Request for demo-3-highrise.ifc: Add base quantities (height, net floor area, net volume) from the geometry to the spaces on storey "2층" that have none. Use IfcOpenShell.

First a look at what the model holds.

```python
import ifcopenshell
import ifcopenshell.util.element
import ifcopenshell.util.unit

model = ifcopenshell.open("demo-3-highrise.ifc")
print(model.schema)
for unit_type in ("LENGTHUNIT", "AREAUNIT", "VOLUMEUNIT"):
    print(unit_type, ifcopenshell.util.unit.calculate_unit_scale(model, unit_type))
storey = next(s for s in model.by_type("IfcBuildingStorey") if s.Name == "2층")
spaces = [e for e in ifcopenshell.util.element.get_decomposition(storey) if e.is_a("IfcSpace")]
for e in sorted(spaces, key=lambda e: e.id()):
    print(e.id(), e.is_a(), e.Name, list(ifcopenshell.util.element.get_psets(e, qtos_only=True)), sep=" | ")
```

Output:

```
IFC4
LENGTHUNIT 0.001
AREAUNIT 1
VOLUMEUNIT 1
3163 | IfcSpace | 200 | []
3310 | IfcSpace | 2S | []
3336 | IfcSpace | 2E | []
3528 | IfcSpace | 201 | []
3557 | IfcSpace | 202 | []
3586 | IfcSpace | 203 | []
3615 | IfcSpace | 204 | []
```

```python
import ifcopenshell
import ifcopenshell.api.pset
import ifcopenshell.geom
import ifcopenshell.util.element
import ifcopenshell.util.shape
import ifcopenshell.util.unit

model = ifcopenshell.open("demo-3-highrise.ifc")
unit_scale = ifcopenshell.util.unit.calculate_unit_scale(model)
area_scale = ifcopenshell.util.unit.calculate_unit_scale(model, "AREAUNIT")
volume_scale = ifcopenshell.util.unit.calculate_unit_scale(model, "VOLUMEUNIT")
settings = ifcopenshell.geom.settings()

storey = next(s for s in model.by_type("IfcBuildingStorey") if s.Name == "2층")
spaces = [e for e in ifcopenshell.util.element.get_decomposition(storey) if e.is_a("IfcSpace")]

for e in sorted(spaces, key=lambda e: e.id()):
    if ifcopenshell.util.element.get_psets(e, qtos_only=True, should_inherit=False):
        continue
    # Geometry comes back in metres, in the element's own axes.
    shape = ifcopenshell.geom.create_shape(settings, e)
    values = {
        "Height": ifcopenshell.util.shape.get_z(shape.geometry) / unit_scale,
        "NetFloorArea": ifcopenshell.util.shape.get_footprint_area(shape.geometry) / area_scale,
        "NetVolume": ifcopenshell.util.shape.get_volume(shape.geometry) / volume_scale,
    }
    qto = ifcopenshell.api.pset.add_qto(model, product=e, name="Qto_SpaceBaseQuantities")
    ifcopenshell.api.pset.edit_qto(model, qto=qto, properties=values)
    print(e.id(), {k: round(v, 3) for k, v in values.items()})

model.write("demo-3-highrise_v2.ifc")
```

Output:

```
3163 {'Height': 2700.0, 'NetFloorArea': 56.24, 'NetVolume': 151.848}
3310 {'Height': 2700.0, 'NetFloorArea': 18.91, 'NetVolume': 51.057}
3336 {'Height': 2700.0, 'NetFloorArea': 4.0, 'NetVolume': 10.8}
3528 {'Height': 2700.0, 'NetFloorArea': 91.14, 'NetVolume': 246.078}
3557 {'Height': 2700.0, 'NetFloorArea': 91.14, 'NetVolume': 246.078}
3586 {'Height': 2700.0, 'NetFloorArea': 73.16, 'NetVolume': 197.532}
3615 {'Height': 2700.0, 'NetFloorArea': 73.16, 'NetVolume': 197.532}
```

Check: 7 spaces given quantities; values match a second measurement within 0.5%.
